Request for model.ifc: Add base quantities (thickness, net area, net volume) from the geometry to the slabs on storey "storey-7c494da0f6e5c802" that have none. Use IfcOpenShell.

First a look at what the model holds.

```python
import ifcopenshell
import ifcopenshell.util.element
import ifcopenshell.util.unit

model = ifcopenshell.open("model.ifc")
print(model.schema)
for unit_type in ("LENGTHUNIT", "AREAUNIT", "VOLUMEUNIT"):
    print(unit_type, ifcopenshell.util.unit.calculate_unit_scale(model, unit_type))
storey = next(s for s in model.by_type("IfcBuildingStorey") if s.Name == "storey-7c494da0f6e5c802")
slabs = [e for e in ifcopenshell.util.element.get_decomposition(storey) if e.is_a("IfcSlab")]
for e in sorted(slabs, key=lambda e: e.id()):
    print(e.id(), e.is_a(), e.Name, list(ifcopenshell.util.element.get_psets(e, qtos_only=True)), sep=" | ")
```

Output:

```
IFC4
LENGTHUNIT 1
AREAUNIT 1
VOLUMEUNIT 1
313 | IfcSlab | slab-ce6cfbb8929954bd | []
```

```python
import ifcopenshell
import ifcopenshell.api.pset
import ifcopenshell.geom
import ifcopenshell.util.element
import ifcopenshell.util.shape
import ifcopenshell.util.unit

model = ifcopenshell.open("model.ifc")
unit_scale = ifcopenshell.util.unit.calculate_unit_scale(model)
area_scale = ifcopenshell.util.unit.calculate_unit_scale(model, "AREAUNIT")
volume_scale = ifcopenshell.util.unit.calculate_unit_scale(model, "VOLUMEUNIT")
settings = ifcopenshell.geom.settings()

storey = next(s for s in model.by_type("IfcBuildingStorey") if s.Name == "storey-7c494da0f6e5c802")
slabs = [e for e in ifcopenshell.util.element.get_decomposition(storey) if e.is_a("IfcSlab")]

for e in sorted(slabs, key=lambda e: e.id()):
    if ifcopenshell.util.element.get_psets(e, qtos_only=True, should_inherit=False):
        continue
    # Geometry comes back in metres, in the element's own axes.
    shape = ifcopenshell.geom.create_shape(settings, e)
    values = {
        "Width": ifcopenshell.util.shape.get_z(shape.geometry) / unit_scale,
        "NetArea": ifcopenshell.util.shape.get_footprint_area(shape.geometry) / area_scale,
        "NetVolume": ifcopenshell.util.shape.get_volume(shape.geometry) / volume_scale,
    }
    qto = ifcopenshell.api.pset.add_qto(model, product=e, name="Qto_SlabBaseQuantities")
    ifcopenshell.api.pset.edit_qto(model, qto=qto, properties=values)
    print(e.id(), {k: round(v, 3) for k, v in values.items()})

model.write("model_updated.ifc")
```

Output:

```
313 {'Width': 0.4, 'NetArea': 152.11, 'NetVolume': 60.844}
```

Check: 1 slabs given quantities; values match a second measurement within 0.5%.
